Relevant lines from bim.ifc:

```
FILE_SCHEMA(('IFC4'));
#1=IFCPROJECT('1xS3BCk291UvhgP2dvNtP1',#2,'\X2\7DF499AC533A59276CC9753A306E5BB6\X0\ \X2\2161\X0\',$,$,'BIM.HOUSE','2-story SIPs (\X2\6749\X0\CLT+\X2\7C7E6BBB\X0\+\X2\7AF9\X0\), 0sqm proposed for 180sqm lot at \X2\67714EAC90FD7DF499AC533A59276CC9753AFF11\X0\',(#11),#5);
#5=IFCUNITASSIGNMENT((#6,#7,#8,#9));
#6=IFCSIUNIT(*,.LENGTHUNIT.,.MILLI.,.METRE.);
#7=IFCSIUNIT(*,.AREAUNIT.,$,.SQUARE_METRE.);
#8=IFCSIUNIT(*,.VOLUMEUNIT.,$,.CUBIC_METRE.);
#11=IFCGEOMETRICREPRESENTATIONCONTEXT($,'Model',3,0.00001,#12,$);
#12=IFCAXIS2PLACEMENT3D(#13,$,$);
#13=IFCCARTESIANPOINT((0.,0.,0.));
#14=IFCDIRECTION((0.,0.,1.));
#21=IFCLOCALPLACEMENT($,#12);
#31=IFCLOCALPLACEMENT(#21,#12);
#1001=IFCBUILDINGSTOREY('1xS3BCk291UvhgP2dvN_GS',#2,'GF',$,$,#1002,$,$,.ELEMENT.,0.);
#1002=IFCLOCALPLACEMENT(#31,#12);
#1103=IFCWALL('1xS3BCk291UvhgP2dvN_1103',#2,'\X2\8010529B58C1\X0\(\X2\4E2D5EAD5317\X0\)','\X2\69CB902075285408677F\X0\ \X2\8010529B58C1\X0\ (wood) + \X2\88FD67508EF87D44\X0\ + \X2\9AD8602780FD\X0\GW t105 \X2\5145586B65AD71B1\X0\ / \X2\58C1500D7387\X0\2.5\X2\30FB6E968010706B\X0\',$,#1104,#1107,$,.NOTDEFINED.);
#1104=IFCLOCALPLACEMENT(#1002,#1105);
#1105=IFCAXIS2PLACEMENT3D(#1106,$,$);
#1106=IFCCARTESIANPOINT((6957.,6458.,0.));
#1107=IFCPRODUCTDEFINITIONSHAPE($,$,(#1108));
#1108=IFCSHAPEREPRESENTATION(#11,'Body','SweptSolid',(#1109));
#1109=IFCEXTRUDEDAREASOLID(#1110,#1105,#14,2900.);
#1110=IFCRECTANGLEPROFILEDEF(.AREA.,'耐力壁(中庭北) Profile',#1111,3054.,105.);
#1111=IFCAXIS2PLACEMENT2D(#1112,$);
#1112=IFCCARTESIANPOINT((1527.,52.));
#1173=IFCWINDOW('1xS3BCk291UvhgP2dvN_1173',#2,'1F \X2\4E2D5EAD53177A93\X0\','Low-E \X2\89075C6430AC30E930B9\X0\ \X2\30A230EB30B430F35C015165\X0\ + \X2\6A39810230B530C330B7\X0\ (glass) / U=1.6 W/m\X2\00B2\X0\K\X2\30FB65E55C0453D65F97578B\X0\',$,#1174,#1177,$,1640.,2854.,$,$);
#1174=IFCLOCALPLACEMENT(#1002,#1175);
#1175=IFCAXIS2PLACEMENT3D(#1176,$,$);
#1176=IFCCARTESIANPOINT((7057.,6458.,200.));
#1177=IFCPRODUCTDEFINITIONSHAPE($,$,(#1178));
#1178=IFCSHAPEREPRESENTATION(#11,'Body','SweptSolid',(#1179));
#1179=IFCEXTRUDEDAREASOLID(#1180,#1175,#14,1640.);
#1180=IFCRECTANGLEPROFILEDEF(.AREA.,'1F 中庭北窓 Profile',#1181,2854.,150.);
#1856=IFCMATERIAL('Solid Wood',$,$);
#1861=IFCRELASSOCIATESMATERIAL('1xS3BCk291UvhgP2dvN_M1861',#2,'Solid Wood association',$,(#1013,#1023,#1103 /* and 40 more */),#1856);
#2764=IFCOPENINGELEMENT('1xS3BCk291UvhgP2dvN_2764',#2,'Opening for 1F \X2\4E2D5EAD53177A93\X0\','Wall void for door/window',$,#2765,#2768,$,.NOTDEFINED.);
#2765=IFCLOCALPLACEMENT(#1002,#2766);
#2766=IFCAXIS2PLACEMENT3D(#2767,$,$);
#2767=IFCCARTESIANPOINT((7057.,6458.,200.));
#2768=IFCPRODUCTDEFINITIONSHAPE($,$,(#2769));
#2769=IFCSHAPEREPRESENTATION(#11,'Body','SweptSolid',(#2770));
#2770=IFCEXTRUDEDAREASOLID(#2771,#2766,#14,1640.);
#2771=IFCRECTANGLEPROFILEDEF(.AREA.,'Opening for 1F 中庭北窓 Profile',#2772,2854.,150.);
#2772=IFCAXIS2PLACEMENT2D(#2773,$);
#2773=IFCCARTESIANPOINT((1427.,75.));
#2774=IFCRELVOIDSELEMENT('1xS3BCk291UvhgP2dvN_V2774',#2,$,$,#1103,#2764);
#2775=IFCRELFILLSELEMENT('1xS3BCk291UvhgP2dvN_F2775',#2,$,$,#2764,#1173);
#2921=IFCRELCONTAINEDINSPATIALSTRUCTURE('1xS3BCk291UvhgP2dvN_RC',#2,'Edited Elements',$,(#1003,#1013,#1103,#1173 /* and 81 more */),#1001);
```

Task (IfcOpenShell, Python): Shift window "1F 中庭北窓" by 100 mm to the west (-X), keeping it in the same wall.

```python
import ifcopenshell
import ifcopenshell.api.geometry
import ifcopenshell.util.placement
import ifcopenshell.util.unit

model = ifcopenshell.open("bim.ifc")
unit_scale = ifcopenshell.util.unit.calculate_unit_scale(model)

window = model.by_guid("1xS3BCk291UvhgP2dvN_1173")
opening = window.FillsVoids[0].RelatingOpeningElement
wall = opening.VoidsElements[0].RelatingBuildingElement

wall_matrix = ifcopenshell.util.placement.get_local_placement(wall.ObjectPlacement)
shift = wall_matrix[:3, 0] * -0.1 / unit_scale
before = ifcopenshell.util.placement.get_local_placement(window.ObjectPlacement)[:3, 3].copy()

# The window is not placed relative to its opening, so move both.
for product in (opening, window):
    matrix = ifcopenshell.util.placement.get_local_placement(product.ObjectPlacement)
    matrix[:3, 3] += shift
    ifcopenshell.api.geometry.edit_object_placement(model, product=product, matrix=matrix, is_si=False)

after = ifcopenshell.util.placement.get_local_placement(window.ObjectPlacement)[:3, 3]
print("window moved by", (after - before).round(3) + 0.0)

model.write("bim_edited.ifc")
```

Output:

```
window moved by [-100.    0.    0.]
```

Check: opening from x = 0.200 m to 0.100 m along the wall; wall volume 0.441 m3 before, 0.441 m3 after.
